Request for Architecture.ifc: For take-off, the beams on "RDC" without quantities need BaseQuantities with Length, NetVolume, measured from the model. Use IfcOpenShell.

First a look at what the model holds.

```python
import ifcopenshell
import ifcopenshell.util.element
import ifcopenshell.util.unit

model = ifcopenshell.open("Architecture.ifc")
print(model.schema)
for unit_type in ("LENGTHUNIT", "AREAUNIT", "VOLUMEUNIT"):
    print(unit_type, ifcopenshell.util.unit.calculate_unit_scale(model, unit_type))
storey = next(s for s in model.by_type("IfcBuildingStorey") if s.Name == "RDC")
beams = [e for e in ifcopenshell.util.element.get_decomposition(storey) if e.is_a("IfcBeam")]
for e in sorted(beams, key=lambda e: e.id()):
    print(e.id(), e.is_a(), e.Name, list(ifcopenshell.util.element.get_psets(e, qtos_only=True)), sep=" | ")
```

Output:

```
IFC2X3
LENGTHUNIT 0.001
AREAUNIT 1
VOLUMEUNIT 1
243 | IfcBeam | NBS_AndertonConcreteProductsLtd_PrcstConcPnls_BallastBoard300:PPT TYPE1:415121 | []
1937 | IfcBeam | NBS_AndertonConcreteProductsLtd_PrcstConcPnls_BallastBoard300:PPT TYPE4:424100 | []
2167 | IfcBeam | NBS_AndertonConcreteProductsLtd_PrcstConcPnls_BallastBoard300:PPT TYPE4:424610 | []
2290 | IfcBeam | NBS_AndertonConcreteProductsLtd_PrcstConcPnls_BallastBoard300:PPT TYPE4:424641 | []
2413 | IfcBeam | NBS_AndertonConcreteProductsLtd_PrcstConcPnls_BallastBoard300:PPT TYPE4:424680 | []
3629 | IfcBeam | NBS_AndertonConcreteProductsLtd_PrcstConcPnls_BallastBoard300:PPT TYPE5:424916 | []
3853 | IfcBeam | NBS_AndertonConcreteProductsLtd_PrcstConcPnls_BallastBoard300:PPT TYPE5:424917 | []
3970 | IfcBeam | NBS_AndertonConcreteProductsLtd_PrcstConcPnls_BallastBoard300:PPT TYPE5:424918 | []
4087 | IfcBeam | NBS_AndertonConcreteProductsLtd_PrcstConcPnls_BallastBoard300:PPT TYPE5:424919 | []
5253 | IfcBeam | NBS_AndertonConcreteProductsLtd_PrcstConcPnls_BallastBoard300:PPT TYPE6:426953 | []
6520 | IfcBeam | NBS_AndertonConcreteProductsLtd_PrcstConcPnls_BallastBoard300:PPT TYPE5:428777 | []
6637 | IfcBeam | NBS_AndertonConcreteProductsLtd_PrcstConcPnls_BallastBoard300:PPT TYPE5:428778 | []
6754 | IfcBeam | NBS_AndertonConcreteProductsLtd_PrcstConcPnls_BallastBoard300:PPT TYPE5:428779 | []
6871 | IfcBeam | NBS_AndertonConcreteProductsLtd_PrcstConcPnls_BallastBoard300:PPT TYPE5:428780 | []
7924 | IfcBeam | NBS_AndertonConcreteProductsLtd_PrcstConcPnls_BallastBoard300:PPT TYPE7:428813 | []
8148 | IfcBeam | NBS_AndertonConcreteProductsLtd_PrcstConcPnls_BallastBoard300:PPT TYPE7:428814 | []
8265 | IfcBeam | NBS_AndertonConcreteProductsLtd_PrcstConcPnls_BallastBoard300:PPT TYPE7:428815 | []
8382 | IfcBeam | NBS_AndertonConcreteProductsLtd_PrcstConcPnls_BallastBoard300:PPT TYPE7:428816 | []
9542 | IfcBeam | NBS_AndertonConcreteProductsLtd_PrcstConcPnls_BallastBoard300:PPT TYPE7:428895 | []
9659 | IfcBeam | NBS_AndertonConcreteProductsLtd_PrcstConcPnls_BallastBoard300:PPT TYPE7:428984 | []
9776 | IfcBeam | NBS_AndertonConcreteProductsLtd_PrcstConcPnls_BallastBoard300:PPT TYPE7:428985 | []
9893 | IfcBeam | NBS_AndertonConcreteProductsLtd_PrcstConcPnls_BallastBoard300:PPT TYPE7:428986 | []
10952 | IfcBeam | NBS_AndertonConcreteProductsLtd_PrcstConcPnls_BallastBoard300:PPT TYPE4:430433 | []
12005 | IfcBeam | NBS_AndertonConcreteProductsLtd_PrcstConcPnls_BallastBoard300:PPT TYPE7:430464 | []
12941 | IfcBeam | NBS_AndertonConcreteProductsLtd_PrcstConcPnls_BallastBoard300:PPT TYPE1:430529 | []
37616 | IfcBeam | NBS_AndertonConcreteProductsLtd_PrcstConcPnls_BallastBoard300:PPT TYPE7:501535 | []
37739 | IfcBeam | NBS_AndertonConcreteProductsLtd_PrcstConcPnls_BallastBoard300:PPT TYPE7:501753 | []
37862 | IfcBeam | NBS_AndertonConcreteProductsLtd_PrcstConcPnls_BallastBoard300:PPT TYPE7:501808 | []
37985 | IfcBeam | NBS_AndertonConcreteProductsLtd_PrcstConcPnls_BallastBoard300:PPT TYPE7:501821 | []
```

```python
import ifcopenshell
import ifcopenshell.api.pset
import ifcopenshell.geom
import ifcopenshell.util.element
import ifcopenshell.util.shape
import ifcopenshell.util.unit

model = ifcopenshell.open("Architecture.ifc")
unit_scale = ifcopenshell.util.unit.calculate_unit_scale(model)
volume_scale = ifcopenshell.util.unit.calculate_unit_scale(model, "VOLUMEUNIT")
settings = ifcopenshell.geom.settings()

storey = next(s for s in model.by_type("IfcBuildingStorey") if s.Name == "RDC")
beams = [e for e in ifcopenshell.util.element.get_decomposition(storey) if e.is_a("IfcBeam")]

for e in sorted(beams, key=lambda e: e.id()):
    if ifcopenshell.util.element.get_psets(e, qtos_only=True, should_inherit=False):
        continue
    # Geometry comes back in metres, in the element's own axes.
    shape = ifcopenshell.geom.create_shape(settings, e)
    values = {
        "Length": ifcopenshell.util.shape.get_max_xyz(shape.geometry) / unit_scale,
        "NetVolume": ifcopenshell.util.shape.get_volume(shape.geometry) / volume_scale,
    }
    qto = ifcopenshell.api.pset.add_qto(model, product=e, name="BaseQuantities")
    ifcopenshell.api.pset.edit_qto(model, qto=qto, properties=values)
    print(e.id(), {k: round(v, 3) for k, v in values.items()})

model.write("Architecture-out.ifc")
```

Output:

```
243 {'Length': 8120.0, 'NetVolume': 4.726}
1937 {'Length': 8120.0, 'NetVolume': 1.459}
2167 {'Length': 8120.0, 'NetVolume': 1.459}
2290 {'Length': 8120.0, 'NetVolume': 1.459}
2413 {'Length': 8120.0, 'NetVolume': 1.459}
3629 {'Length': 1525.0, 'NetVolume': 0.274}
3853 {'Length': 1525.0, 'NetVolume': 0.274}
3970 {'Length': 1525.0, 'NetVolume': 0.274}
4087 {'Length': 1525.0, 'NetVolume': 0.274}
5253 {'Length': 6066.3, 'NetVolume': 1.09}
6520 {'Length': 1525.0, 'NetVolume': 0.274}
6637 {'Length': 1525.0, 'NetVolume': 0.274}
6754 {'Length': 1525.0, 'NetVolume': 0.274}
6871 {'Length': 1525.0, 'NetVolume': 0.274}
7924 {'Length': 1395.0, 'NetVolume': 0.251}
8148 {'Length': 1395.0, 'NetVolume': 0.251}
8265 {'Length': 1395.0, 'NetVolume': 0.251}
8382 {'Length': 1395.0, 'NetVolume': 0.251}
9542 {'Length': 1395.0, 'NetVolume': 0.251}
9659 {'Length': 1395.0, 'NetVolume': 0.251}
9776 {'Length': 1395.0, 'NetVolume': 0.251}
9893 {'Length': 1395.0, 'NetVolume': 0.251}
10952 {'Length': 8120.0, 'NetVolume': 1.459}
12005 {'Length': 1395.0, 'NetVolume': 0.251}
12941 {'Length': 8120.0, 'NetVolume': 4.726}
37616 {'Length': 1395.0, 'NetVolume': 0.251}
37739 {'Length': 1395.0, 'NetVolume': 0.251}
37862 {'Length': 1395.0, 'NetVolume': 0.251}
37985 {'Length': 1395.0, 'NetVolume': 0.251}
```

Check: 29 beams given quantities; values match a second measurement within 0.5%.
